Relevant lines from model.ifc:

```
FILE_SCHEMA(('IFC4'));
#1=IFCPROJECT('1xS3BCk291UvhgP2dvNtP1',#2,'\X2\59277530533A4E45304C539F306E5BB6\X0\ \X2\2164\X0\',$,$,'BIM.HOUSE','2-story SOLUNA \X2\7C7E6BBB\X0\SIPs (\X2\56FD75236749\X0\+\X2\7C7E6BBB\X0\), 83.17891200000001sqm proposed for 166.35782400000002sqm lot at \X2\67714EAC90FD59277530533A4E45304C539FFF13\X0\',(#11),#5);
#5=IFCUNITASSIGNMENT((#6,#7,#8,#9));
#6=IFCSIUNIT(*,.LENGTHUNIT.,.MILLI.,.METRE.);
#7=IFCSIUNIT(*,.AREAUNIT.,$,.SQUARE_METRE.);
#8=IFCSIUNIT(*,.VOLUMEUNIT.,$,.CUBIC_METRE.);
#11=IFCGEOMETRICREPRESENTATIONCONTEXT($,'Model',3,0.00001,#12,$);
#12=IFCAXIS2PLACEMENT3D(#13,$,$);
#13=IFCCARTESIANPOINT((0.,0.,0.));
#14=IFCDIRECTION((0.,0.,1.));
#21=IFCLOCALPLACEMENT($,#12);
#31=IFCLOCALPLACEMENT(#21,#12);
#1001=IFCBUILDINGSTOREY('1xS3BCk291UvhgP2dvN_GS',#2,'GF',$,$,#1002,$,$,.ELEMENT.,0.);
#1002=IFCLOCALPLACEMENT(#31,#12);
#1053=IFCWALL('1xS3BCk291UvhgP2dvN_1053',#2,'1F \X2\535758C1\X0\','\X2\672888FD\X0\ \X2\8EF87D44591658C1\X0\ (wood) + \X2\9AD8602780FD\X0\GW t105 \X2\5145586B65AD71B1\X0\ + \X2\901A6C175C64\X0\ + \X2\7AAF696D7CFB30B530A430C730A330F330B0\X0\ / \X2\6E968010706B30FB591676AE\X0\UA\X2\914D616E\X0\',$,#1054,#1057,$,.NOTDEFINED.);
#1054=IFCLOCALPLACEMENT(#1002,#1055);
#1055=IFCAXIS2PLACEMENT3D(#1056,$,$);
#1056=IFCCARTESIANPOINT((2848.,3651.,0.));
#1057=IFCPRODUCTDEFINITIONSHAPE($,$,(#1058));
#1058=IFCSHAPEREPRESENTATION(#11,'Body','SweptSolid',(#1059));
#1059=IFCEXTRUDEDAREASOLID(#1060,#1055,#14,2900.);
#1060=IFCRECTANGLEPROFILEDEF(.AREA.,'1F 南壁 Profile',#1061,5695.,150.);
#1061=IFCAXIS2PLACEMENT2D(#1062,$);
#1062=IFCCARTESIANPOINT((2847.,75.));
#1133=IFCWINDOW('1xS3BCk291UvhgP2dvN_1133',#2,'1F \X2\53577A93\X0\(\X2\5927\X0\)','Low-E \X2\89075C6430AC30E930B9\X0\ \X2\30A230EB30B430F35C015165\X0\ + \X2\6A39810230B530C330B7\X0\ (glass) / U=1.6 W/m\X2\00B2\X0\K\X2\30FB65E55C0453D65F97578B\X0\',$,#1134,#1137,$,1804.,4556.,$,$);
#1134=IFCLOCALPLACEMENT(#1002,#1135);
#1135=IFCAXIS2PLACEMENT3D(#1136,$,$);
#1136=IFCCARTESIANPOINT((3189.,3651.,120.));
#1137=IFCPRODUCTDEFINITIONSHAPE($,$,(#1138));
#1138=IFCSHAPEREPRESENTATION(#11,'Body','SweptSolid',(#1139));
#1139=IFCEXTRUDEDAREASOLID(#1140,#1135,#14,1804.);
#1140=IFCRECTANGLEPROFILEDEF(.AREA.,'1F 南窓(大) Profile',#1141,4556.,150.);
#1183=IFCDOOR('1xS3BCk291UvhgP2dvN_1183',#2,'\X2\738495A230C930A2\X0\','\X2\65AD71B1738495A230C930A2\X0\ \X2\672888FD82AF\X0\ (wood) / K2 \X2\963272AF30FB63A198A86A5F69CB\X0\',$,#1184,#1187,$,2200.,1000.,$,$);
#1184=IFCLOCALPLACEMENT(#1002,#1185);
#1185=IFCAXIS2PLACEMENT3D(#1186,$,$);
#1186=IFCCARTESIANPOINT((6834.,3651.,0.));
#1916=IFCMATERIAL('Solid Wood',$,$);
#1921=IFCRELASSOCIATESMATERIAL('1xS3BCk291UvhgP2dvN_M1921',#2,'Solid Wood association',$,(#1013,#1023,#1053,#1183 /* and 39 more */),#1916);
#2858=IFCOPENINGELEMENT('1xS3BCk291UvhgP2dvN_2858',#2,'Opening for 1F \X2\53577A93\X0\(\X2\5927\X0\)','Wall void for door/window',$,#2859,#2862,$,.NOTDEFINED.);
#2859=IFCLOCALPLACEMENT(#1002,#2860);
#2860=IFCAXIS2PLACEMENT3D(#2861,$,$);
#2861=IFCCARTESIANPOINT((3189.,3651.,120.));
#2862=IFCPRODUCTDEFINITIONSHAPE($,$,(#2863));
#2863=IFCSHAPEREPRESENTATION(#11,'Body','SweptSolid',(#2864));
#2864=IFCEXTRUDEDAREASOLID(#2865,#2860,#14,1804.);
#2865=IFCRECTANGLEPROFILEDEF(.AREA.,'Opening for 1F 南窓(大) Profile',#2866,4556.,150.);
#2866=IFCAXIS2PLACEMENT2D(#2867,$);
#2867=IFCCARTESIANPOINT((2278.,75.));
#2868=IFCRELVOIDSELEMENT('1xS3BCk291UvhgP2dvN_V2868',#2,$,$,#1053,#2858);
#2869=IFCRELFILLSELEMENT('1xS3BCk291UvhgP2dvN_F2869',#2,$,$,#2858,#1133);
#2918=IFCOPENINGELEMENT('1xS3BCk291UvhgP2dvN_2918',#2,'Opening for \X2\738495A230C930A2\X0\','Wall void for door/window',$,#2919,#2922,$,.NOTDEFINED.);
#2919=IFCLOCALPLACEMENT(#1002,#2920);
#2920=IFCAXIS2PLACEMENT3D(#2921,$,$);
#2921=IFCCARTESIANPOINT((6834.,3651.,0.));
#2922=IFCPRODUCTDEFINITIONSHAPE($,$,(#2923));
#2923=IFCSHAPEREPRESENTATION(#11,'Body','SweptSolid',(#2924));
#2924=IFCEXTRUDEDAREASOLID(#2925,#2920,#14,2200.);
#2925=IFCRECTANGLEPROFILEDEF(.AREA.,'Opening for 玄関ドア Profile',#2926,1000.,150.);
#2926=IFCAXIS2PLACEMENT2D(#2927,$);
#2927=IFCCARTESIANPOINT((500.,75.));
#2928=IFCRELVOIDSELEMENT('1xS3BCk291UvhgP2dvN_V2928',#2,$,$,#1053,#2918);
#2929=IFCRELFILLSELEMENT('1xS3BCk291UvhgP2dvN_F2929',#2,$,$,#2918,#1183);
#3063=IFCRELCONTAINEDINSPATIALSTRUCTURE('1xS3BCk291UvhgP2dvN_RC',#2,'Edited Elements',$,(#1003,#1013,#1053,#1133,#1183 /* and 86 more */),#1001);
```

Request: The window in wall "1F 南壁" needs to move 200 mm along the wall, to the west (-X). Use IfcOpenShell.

```python
import ifcopenshell
import ifcopenshell.api.geometry
import ifcopenshell.util.placement
import ifcopenshell.util.unit

model = ifcopenshell.open("model.ifc")
unit_scale = ifcopenshell.util.unit.calculate_unit_scale(model)

window = model.by_guid("1xS3BCk291UvhgP2dvN_1133")
opening = window.FillsVoids[0].RelatingOpeningElement
wall = opening.VoidsElements[0].RelatingBuildingElement

wall_matrix = ifcopenshell.util.placement.get_local_placement(wall.ObjectPlacement)
shift = wall_matrix[:3, 0] * -0.2 / unit_scale
before = ifcopenshell.util.placement.get_local_placement(window.ObjectPlacement)[:3, 3].copy()

# The window is not placed relative to its opening, so move both.
for product in (opening, window):
    matrix = ifcopenshell.util.placement.get_local_placement(product.ObjectPlacement)
    matrix[:3, 3] += shift
    ifcopenshell.api.geometry.edit_object_placement(model, product=product, matrix=matrix, is_si=False)

after = ifcopenshell.util.placement.get_local_placement(window.ObjectPlacement)[:3, 3]
print("window moved by", (after - before).round(3) + 0.0)

model.write("model_v2.ifc")
```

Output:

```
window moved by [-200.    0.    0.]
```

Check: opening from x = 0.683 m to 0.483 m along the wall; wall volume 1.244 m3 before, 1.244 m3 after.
